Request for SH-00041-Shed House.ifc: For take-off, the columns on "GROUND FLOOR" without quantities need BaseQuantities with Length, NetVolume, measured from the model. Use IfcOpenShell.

First a look at what the model holds.

```python
import ifcopenshell
import ifcopenshell.util.element
import ifcopenshell.util.unit

model = ifcopenshell.open("SH-00041-Shed House.ifc")
print(model.schema)
for unit_type in ("LENGTHUNIT", "AREAUNIT", "VOLUMEUNIT"):
    print(unit_type, ifcopenshell.util.unit.calculate_unit_scale(model, unit_type))
storey = next(s for s in model.by_type("IfcBuildingStorey") if s.Name == "GROUND FLOOR")
columns = [e for e in ifcopenshell.util.element.get_decomposition(storey) if e.is_a("IfcColumn")]
for e in sorted(columns, key=lambda e: e.id()):
    print(e.id(), e.is_a(), e.Name, list(ifcopenshell.util.element.get_psets(e, qtos_only=True)), sep=" | ")
```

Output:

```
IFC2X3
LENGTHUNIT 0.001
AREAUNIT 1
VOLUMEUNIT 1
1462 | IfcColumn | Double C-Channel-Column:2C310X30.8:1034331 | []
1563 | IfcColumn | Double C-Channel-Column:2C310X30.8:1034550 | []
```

```python
import ifcopenshell
import ifcopenshell.api.pset
import ifcopenshell.geom
import ifcopenshell.util.element
import ifcopenshell.util.shape
import ifcopenshell.util.unit

model = ifcopenshell.open("SH-00041-Shed House.ifc")
unit_scale = ifcopenshell.util.unit.calculate_unit_scale(model)
volume_scale = ifcopenshell.util.unit.calculate_unit_scale(model, "VOLUMEUNIT")
settings = ifcopenshell.geom.settings()

storey = next(s for s in model.by_type("IfcBuildingStorey") if s.Name == "GROUND FLOOR")
columns = [e for e in ifcopenshell.util.element.get_decomposition(storey) if e.is_a("IfcColumn")]

for e in sorted(columns, key=lambda e: e.id()):
    if ifcopenshell.util.element.get_psets(e, qtos_only=True, should_inherit=False):
        continue
    # Geometry comes back in metres, in the element's own axes.
    shape = ifcopenshell.geom.create_shape(settings, e)
    values = {
        "Length": ifcopenshell.util.shape.get_z(shape.geometry) / unit_scale,
        "NetVolume": ifcopenshell.util.shape.get_volume(shape.geometry) / volume_scale,
    }
    qto = ifcopenshell.api.pset.add_qto(model, product=e, name="BaseQuantities")
    ifcopenshell.api.pset.edit_qto(model, qto=qto, properties=values)
    print(e.id(), {k: round(v, 3) for k, v in values.items()})

model.write("SH-00041-Shed House_updated.ifc")
```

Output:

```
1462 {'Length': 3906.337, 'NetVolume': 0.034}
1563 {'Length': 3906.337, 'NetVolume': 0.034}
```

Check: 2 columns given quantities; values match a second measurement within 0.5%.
